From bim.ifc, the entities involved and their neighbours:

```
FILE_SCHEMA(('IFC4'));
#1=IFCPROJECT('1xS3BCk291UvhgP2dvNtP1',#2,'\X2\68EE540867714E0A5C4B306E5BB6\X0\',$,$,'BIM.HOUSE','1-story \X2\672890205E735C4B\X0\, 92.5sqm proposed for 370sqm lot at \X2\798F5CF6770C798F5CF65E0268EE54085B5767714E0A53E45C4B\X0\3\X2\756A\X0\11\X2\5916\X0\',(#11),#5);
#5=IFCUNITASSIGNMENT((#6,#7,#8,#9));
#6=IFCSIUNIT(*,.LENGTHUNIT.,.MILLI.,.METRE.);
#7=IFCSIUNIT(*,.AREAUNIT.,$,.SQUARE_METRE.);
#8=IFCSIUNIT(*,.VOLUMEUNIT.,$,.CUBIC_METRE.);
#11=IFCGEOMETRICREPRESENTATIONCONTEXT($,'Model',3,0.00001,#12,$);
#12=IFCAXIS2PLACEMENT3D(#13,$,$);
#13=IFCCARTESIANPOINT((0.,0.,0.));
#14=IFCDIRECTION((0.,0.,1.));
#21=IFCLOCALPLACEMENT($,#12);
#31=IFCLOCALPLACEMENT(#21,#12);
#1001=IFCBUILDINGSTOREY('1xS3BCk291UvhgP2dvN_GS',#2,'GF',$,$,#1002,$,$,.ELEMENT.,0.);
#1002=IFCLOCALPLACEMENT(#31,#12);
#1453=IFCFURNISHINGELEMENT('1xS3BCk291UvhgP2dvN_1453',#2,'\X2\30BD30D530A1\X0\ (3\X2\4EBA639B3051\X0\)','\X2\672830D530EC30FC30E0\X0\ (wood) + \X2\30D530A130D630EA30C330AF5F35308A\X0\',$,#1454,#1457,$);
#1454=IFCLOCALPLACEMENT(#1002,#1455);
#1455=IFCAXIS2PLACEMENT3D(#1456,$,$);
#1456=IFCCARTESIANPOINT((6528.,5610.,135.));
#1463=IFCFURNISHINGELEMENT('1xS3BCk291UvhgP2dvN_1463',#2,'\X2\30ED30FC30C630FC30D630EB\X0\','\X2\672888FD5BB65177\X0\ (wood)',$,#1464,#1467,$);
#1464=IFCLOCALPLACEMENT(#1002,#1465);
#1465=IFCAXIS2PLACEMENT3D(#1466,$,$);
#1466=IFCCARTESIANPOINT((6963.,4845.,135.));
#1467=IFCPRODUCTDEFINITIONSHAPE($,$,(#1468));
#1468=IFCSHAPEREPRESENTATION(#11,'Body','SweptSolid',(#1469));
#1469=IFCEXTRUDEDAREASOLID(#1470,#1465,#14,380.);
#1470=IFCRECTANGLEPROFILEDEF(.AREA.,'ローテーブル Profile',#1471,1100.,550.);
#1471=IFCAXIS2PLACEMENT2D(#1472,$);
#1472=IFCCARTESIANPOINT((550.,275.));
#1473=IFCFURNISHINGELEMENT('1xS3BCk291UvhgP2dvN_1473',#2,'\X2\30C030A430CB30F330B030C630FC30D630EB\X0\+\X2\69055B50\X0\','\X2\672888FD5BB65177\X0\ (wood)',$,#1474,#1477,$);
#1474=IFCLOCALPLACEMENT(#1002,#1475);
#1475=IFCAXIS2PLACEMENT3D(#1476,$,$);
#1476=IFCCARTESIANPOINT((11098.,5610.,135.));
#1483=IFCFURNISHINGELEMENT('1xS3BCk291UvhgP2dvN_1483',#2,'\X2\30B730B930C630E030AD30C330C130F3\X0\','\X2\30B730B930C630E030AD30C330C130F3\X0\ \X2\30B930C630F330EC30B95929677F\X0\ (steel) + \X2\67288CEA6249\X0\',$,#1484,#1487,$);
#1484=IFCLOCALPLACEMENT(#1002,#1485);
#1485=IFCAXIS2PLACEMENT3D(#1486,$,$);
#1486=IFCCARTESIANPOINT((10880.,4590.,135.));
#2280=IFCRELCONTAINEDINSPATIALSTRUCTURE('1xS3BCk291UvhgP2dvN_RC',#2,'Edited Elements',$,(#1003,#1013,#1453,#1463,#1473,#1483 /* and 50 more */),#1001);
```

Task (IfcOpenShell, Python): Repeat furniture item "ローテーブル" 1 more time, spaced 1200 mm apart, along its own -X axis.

```python
import ifcopenshell
import ifcopenshell.api.geometry
import ifcopenshell.api.root
import ifcopenshell.util.element
import ifcopenshell.util.placement
import ifcopenshell.util.unit

model = ifcopenshell.open("bim.ifc")
unit_scale = ifcopenshell.util.unit.calculate_unit_scale(model)


def reuse_history(source, copy):
    """copy_class also copies each property set's owner history, people and application; keep the originals."""
    for rel in copy.IsDefinedBy:
        if rel.is_a("IfcRelDefinesByProperties") and (history := rel.RelatingPropertyDefinition.OwnerHistory):
            rel.RelatingPropertyDefinition.OwnerHistory = source.OwnerHistory
            ifcopenshell.util.element.remove_deep2(model, history)


source = model.by_id(1463)
base = ifcopenshell.util.placement.get_local_placement(source.ObjectPlacement)
step = -base[:3, 0] * 1.2 / unit_scale

for i in range(1, 2):
    copy = ifcopenshell.api.root.copy_class(model, product=source)
    copy.Representation = ifcopenshell.util.element.copy_deep(
        model, source.Representation, exclude=["IfcGeometricRepresentationContext", "IfcRepresentationMap"]
    )
    reuse_history(source, copy)
    matrix = base.copy()
    matrix[:3, 3] += i * step
    print("added at", matrix[:3, 3].round(3) + 0.0)
    ifcopenshell.api.geometry.edit_object_placement(model, product=copy, matrix=matrix, is_si=False)

model.write("bim_rev.ifc")
```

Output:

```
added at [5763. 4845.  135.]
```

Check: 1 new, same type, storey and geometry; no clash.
